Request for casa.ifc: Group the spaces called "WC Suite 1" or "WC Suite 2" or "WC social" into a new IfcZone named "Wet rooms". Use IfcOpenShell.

First a look at what the model holds.

```python
import ifcopenshell

model = ifcopenshell.open("casa.ifc")
print(model.schema)
seen = {}
for space in model.by_type("IfcSpace"):
    seen[space.Name] = seen.get(space.Name, 0) + 1
for name, count in sorted(seen.items(), key=str):
    print(count, "x", name)
print("zones:", [z.Name for z in model.by_type("IfcZone")][:20])
```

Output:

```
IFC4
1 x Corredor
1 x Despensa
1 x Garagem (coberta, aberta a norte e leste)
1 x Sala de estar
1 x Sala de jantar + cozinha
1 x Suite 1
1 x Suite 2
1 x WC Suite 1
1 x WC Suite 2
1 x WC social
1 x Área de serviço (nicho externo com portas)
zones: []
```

```python
import ifcopenshell
import ifcopenshell.api.group
import ifcopenshell.api.root

model = ifcopenshell.open("casa.ifc")

names = {"WC Suite 1", "WC Suite 2", "WC social"}
spaces = [s for s in model.by_type("IfcSpace") if s.Name in names]

zone = ifcopenshell.api.root.create_entity(model, ifc_class="IfcZone", name="Wet rooms")
ifcopenshell.api.group.assign_group(model, products=spaces, group=zone)
print(len(spaces), "spaces in", zone.Name)

model.write("casa_rev.ifc")
```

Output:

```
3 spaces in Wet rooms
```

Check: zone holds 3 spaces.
